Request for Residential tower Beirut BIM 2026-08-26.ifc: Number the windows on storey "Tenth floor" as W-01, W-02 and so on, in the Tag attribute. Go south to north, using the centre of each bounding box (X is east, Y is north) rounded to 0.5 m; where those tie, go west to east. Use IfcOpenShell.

First a look at what the model holds.

```python
import ifcopenshell
import ifcopenshell.util.element
import ifcopenshell.util.placement

model = ifcopenshell.open("Residential tower Beirut BIM 2026-08-26.ifc")
print(model.schema)
storey = next(s for s in model.by_type("IfcBuildingStorey") if s.Name == "Tenth floor")
windows = [e for e in ifcopenshell.util.element.get_decomposition(storey) if e.is_a("IfcWindow")]
for e in sorted(windows, key=lambda e: e.id()):
    origin = ifcopenshell.util.placement.get_local_placement(e.ObjectPlacement)[:3, 3]
    print(e.id(), e.Tag, e.Name, origin.round(2) + 0.0, sep=" | ")
```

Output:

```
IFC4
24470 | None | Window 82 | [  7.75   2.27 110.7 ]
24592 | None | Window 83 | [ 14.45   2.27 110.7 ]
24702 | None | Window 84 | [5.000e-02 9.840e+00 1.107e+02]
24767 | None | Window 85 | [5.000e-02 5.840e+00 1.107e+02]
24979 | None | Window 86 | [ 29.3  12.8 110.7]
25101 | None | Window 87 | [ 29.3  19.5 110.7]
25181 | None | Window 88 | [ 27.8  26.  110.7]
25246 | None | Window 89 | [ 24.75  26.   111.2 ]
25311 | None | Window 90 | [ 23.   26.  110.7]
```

```python
import ifcopenshell
import ifcopenshell.geom
import ifcopenshell.util.element
import ifcopenshell.util.shape

model = ifcopenshell.open("Residential tower Beirut BIM 2026-08-26.ifc")
settings = ifcopenshell.geom.settings()
settings.set("use-world-coords", True)


def centre(element):
    shape = ifcopenshell.geom.create_shape(settings, element)
    return ifcopenshell.util.shape.get_bbox_centroid(shape.geometry)


storey = next(s for s in model.by_type("IfcBuildingStorey") if s.Name == "Tenth floor")
windows = [e for e in ifcopenshell.util.element.get_decomposition(storey) if e.is_a("IfcWindow")]

# Insertion points can sit at a corner or the storey origin, so sort by the geometry (in metres).
centres = {e: centre(e) for e in windows}
windows.sort(key=lambda e: (round(centres[e][1] / 0.5), centres[e][0]))

for i, e in enumerate(windows, start=1):
    number = f"W-{i:02d}"
    e.Tag = number
    print(e.id(), number)

model.write("Residential tower Beirut BIM 2026-08-26_v2.ifc")
```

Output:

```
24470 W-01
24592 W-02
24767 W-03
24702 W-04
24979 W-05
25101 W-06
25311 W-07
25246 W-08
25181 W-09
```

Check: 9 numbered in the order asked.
